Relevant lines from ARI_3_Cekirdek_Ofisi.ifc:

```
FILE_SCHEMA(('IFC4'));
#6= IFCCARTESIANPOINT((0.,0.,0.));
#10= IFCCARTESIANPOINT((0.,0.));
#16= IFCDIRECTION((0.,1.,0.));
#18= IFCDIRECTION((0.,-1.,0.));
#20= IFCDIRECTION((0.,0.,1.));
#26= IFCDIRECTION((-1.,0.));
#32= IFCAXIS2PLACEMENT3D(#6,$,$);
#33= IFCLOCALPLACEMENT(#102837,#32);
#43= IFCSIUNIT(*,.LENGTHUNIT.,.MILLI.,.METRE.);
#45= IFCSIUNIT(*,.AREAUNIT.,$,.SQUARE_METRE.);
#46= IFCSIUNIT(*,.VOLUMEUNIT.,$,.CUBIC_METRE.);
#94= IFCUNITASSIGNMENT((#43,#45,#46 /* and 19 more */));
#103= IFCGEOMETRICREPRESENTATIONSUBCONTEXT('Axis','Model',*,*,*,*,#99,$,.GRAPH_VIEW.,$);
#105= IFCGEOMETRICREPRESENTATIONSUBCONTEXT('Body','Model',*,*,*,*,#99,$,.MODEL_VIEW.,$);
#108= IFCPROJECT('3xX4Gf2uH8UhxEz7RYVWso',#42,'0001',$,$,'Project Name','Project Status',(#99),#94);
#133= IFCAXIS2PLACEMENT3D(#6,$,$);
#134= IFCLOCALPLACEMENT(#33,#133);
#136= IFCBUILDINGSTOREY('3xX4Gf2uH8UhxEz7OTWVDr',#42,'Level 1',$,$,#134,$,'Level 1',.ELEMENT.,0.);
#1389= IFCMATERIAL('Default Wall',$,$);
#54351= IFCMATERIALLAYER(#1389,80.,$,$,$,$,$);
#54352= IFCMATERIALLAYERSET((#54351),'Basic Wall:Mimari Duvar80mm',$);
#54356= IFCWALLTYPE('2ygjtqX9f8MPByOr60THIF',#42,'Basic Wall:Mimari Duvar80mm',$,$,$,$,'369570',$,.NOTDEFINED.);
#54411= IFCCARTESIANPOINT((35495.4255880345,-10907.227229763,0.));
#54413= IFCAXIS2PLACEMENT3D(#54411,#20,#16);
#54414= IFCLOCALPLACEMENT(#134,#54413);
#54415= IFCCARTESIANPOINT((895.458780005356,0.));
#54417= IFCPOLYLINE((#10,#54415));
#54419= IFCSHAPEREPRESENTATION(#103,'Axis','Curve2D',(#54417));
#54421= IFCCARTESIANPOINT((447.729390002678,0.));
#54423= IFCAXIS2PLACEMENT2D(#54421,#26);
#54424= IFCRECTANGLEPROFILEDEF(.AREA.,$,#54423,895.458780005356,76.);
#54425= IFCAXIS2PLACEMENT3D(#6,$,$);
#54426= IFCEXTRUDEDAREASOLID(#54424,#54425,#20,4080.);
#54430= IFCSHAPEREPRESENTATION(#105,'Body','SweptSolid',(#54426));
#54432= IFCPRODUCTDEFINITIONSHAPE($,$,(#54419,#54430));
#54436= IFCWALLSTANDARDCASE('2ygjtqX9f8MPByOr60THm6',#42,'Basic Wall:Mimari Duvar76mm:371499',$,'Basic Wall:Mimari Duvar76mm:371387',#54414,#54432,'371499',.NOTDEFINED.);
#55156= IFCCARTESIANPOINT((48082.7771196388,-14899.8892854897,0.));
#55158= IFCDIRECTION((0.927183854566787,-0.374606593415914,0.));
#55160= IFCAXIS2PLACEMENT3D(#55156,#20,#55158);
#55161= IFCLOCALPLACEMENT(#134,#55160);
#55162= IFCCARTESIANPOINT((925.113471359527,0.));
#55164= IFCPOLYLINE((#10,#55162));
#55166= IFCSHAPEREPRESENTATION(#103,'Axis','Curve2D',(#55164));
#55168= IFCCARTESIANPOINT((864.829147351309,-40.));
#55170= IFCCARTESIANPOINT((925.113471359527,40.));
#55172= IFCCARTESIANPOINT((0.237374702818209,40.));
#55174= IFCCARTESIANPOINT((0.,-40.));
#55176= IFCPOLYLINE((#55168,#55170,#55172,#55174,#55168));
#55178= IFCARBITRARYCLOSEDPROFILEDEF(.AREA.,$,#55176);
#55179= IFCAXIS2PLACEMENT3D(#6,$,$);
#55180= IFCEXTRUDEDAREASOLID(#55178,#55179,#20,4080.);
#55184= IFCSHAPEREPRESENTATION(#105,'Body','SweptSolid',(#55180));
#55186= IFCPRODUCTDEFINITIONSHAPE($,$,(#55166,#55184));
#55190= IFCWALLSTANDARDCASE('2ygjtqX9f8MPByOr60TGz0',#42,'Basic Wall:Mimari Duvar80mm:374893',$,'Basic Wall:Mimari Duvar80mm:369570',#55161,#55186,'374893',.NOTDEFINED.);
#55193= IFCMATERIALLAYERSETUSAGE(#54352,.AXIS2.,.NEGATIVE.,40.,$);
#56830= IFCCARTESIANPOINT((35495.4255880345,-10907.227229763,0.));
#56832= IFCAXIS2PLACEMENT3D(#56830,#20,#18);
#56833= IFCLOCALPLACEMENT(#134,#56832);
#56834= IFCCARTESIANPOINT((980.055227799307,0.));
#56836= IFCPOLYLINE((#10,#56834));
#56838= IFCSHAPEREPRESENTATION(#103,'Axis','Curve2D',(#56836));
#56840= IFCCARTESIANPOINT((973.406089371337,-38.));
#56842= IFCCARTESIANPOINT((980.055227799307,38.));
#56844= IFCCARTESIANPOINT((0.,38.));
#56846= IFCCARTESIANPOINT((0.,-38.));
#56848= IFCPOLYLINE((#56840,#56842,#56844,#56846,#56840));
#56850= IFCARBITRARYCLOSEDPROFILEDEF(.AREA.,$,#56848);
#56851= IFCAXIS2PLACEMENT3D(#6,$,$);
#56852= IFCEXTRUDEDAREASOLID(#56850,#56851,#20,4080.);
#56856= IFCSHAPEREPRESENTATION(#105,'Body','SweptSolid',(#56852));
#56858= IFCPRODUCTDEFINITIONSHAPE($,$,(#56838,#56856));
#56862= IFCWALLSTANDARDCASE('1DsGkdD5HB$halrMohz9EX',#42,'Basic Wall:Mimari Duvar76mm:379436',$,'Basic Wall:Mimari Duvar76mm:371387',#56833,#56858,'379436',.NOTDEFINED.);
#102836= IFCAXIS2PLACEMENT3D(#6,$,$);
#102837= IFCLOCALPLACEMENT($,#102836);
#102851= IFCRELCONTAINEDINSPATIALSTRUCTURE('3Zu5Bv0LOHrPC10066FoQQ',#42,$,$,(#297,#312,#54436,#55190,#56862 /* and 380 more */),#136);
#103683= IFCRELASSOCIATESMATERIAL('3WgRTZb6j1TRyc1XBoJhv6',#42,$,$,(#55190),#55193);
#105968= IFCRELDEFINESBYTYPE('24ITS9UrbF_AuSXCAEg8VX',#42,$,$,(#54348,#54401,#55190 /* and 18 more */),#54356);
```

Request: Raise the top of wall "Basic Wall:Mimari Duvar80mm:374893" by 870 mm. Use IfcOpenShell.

```python
import ifcopenshell
import ifcopenshell.geom
import ifcopenshell.util.representation
import ifcopenshell.util.shape
import ifcopenshell.util.unit

model = ifcopenshell.open("ARI_3_Cekirdek_Ofisi.ifc")
unit_scale = ifcopenshell.util.unit.calculate_unit_scale(model)
settings = ifcopenshell.geom.settings()


def volume(element):
    """Net volume in cubic metres, openings subtracted."""
    shape = ifcopenshell.geom.create_shape(settings, element)
    return ifcopenshell.util.shape.get_volume(shape.geometry)


wall = model.by_guid("2ygjtqX9f8MPByOr60TGz0")
before = volume(wall)

body = ifcopenshell.util.representation.get_representation(wall, "Model", "Body")
solid = body.Items[0]
old_height = solid.Depth
solid.Depth += 0.87 / unit_scale
after = volume(wall)

print(f"height {old_height:g} -> {solid.Depth:g}, volume {before:.3f} -> {after:.3f} m3")

model.write("ARI_3_Cekirdek_Ofisi-out.ifc")
```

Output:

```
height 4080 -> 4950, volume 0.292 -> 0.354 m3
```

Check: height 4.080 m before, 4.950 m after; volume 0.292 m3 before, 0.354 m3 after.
